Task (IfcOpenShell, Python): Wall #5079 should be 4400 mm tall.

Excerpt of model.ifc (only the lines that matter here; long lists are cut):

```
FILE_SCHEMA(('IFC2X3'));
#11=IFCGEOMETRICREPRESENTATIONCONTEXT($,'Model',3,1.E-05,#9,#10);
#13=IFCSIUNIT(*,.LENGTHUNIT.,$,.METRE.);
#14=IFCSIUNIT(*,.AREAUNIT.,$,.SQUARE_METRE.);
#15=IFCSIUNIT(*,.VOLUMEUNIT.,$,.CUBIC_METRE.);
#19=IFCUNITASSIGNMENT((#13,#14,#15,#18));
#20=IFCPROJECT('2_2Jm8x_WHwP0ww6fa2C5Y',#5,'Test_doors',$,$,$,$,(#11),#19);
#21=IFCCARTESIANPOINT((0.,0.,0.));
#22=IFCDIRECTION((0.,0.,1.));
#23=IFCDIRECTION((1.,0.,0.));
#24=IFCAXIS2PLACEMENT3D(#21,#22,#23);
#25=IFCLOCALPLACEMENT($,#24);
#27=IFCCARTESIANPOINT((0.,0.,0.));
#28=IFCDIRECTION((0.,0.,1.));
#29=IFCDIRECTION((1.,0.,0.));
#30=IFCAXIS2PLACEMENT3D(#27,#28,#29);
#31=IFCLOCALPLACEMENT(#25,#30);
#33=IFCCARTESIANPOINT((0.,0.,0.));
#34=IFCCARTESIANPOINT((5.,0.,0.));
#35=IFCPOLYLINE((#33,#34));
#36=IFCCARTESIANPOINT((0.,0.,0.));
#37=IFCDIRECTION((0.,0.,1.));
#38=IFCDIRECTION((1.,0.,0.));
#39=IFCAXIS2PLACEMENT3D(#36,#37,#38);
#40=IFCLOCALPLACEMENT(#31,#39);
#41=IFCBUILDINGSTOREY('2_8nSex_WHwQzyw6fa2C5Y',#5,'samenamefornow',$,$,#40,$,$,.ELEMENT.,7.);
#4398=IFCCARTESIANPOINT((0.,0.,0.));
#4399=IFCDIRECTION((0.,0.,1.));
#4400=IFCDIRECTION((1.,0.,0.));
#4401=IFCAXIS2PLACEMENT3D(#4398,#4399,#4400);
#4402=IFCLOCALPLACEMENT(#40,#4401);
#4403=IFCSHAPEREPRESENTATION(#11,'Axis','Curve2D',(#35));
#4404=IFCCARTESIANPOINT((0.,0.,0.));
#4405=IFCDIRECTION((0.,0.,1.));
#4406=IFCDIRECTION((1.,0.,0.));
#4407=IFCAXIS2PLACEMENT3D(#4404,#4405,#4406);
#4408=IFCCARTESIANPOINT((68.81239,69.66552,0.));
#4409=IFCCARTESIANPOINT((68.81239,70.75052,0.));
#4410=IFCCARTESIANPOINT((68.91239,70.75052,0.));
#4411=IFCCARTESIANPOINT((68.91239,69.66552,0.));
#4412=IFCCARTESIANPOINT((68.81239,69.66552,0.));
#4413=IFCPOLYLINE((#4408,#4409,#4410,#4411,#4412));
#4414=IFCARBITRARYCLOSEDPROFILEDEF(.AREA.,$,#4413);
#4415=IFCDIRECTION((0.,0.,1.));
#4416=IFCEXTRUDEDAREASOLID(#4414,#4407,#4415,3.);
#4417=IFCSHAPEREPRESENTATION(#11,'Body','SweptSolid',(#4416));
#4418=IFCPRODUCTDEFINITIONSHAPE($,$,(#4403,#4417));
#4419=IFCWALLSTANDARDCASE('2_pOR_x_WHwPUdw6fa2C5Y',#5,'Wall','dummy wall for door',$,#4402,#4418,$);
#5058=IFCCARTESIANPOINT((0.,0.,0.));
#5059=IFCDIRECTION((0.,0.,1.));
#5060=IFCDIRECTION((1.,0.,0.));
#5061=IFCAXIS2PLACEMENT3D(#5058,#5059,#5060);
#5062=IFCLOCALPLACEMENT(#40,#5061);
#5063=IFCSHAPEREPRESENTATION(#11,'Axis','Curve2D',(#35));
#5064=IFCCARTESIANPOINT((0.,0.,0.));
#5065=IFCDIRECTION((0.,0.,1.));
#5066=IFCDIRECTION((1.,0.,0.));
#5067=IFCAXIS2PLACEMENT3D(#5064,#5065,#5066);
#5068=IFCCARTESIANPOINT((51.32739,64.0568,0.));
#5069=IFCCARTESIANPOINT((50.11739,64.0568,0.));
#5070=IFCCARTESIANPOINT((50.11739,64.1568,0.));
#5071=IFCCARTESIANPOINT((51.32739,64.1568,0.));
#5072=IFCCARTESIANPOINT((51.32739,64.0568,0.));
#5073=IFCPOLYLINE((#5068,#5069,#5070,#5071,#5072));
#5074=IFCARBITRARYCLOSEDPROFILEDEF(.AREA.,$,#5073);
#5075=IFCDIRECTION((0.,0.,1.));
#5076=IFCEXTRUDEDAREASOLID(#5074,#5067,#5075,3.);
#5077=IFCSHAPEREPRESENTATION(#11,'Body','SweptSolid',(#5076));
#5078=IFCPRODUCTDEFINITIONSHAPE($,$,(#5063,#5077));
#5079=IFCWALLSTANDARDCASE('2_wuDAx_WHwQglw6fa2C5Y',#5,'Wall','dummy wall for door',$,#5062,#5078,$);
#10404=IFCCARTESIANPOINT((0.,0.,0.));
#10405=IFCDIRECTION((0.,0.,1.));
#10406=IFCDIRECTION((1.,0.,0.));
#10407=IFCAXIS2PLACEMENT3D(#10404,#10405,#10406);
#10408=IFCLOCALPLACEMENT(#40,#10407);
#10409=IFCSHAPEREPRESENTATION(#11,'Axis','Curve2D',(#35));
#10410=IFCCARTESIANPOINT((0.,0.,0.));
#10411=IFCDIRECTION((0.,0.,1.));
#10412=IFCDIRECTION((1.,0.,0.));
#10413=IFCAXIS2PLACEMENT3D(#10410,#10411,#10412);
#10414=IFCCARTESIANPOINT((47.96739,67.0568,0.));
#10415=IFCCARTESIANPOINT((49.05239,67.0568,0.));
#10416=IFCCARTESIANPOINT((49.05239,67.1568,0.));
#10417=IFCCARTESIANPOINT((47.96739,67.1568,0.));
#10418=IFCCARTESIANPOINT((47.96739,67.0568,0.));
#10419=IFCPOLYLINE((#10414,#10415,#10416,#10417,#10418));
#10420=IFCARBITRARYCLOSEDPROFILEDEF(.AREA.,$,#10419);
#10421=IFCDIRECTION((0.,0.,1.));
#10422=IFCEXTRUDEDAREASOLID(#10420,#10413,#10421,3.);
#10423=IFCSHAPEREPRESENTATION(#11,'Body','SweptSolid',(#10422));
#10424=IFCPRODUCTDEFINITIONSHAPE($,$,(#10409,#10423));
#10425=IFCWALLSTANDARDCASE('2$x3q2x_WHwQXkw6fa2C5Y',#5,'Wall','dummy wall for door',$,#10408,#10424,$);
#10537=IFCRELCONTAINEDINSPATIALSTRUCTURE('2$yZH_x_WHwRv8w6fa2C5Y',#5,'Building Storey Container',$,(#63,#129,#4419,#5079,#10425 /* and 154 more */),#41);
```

```python
import ifcopenshell
import ifcopenshell.geom
import ifcopenshell.util.shape
import ifcopenshell.util.unit

model = ifcopenshell.open("model.ifc")
unit_scale = ifcopenshell.util.unit.calculate_unit_scale(model)
settings = ifcopenshell.geom.settings()


def volume(element):
    """Net volume in cubic metres, openings subtracted."""
    shape = ifcopenshell.geom.create_shape(settings, element)
    return ifcopenshell.util.shape.get_volume(shape.geometry)


wall = model.by_id(5079)
before = volume(wall)

body = next(r for r in wall.Representation.Representations if r.RepresentationIdentifier == "Body")
solid = body.Items[0]
old_height = solid.Depth
solid.Depth = 4.4 / unit_scale
after = volume(wall)

print(f"height {old_height:g} -> {solid.Depth:g}, volume {before:.3f} -> {after:.3f} m3")

model.write("model_rev.ifc")
```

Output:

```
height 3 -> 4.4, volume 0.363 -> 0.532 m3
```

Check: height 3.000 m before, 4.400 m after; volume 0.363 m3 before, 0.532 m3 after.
